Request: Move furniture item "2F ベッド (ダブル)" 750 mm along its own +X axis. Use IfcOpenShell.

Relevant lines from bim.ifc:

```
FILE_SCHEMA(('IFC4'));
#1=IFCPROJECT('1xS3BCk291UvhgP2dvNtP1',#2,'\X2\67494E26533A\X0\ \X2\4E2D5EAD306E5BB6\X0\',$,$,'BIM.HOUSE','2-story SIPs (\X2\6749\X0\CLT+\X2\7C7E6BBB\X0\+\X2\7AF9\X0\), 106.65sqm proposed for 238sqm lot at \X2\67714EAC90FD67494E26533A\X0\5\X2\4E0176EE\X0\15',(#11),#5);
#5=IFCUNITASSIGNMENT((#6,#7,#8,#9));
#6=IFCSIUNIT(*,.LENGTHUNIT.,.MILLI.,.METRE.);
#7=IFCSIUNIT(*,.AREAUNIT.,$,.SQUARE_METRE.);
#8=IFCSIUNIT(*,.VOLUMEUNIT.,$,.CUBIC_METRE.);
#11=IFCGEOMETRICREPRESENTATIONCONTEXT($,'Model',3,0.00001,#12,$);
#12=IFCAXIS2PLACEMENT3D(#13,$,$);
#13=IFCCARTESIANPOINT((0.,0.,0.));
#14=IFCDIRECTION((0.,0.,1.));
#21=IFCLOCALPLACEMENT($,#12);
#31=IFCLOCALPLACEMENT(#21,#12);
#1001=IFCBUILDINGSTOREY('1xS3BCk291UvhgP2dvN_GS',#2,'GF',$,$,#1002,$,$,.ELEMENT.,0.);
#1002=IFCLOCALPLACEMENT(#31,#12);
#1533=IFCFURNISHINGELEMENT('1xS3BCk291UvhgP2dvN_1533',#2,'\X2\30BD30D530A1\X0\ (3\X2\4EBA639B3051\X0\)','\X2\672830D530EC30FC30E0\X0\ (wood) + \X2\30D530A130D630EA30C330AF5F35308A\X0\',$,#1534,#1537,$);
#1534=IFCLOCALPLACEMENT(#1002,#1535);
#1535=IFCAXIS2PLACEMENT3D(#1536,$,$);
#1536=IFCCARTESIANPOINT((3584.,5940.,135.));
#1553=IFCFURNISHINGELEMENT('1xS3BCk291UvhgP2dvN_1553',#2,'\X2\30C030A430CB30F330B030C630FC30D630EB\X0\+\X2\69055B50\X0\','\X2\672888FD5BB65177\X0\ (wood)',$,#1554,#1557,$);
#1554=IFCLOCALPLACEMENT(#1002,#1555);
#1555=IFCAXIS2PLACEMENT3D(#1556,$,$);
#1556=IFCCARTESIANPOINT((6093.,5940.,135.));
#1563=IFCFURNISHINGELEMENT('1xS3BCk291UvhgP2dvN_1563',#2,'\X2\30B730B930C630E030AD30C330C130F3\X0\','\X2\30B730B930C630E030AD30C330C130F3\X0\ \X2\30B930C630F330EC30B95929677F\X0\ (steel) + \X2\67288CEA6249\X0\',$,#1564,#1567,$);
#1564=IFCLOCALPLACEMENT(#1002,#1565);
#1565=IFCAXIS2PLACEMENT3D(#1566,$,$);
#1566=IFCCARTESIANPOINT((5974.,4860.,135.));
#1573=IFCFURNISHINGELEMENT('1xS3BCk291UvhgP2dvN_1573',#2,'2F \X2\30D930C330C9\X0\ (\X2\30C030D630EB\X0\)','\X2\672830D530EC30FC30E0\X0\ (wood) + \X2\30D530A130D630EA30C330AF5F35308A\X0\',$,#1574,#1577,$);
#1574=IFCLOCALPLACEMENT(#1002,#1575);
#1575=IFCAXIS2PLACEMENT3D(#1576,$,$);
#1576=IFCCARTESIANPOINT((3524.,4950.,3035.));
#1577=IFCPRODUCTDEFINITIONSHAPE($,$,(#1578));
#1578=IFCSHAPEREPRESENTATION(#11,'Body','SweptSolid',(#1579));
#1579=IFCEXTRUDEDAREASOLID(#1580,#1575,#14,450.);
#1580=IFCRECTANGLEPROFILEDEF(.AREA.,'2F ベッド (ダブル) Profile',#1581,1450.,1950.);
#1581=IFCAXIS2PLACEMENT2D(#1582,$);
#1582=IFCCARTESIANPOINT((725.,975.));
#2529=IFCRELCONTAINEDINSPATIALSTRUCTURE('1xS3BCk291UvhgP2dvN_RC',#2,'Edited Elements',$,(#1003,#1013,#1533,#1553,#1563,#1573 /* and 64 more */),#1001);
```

```python
import ifcopenshell
import ifcopenshell.api.geometry
import ifcopenshell.util.placement
import ifcopenshell.util.unit

model = ifcopenshell.open("bim.ifc")
unit_scale = ifcopenshell.util.unit.calculate_unit_scale(model)

item = model.by_guid("1xS3BCk291UvhgP2dvN_1573")
matrix = ifcopenshell.util.placement.get_local_placement(item.ObjectPlacement)
matrix[:3, 3] += matrix[:3, 0] * 0.75 / unit_scale
ifcopenshell.api.geometry.edit_object_placement(model, product=item, matrix=matrix, is_si=False)

print(ifcopenshell.util.placement.get_local_placement(item.ObjectPlacement).round(3) + 0.0)

model.write("bim_rev.ifc")
```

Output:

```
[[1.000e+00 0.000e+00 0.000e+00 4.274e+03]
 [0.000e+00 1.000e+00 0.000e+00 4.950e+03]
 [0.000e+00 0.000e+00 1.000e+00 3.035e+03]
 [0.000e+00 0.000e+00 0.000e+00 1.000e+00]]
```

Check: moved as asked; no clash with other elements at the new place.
